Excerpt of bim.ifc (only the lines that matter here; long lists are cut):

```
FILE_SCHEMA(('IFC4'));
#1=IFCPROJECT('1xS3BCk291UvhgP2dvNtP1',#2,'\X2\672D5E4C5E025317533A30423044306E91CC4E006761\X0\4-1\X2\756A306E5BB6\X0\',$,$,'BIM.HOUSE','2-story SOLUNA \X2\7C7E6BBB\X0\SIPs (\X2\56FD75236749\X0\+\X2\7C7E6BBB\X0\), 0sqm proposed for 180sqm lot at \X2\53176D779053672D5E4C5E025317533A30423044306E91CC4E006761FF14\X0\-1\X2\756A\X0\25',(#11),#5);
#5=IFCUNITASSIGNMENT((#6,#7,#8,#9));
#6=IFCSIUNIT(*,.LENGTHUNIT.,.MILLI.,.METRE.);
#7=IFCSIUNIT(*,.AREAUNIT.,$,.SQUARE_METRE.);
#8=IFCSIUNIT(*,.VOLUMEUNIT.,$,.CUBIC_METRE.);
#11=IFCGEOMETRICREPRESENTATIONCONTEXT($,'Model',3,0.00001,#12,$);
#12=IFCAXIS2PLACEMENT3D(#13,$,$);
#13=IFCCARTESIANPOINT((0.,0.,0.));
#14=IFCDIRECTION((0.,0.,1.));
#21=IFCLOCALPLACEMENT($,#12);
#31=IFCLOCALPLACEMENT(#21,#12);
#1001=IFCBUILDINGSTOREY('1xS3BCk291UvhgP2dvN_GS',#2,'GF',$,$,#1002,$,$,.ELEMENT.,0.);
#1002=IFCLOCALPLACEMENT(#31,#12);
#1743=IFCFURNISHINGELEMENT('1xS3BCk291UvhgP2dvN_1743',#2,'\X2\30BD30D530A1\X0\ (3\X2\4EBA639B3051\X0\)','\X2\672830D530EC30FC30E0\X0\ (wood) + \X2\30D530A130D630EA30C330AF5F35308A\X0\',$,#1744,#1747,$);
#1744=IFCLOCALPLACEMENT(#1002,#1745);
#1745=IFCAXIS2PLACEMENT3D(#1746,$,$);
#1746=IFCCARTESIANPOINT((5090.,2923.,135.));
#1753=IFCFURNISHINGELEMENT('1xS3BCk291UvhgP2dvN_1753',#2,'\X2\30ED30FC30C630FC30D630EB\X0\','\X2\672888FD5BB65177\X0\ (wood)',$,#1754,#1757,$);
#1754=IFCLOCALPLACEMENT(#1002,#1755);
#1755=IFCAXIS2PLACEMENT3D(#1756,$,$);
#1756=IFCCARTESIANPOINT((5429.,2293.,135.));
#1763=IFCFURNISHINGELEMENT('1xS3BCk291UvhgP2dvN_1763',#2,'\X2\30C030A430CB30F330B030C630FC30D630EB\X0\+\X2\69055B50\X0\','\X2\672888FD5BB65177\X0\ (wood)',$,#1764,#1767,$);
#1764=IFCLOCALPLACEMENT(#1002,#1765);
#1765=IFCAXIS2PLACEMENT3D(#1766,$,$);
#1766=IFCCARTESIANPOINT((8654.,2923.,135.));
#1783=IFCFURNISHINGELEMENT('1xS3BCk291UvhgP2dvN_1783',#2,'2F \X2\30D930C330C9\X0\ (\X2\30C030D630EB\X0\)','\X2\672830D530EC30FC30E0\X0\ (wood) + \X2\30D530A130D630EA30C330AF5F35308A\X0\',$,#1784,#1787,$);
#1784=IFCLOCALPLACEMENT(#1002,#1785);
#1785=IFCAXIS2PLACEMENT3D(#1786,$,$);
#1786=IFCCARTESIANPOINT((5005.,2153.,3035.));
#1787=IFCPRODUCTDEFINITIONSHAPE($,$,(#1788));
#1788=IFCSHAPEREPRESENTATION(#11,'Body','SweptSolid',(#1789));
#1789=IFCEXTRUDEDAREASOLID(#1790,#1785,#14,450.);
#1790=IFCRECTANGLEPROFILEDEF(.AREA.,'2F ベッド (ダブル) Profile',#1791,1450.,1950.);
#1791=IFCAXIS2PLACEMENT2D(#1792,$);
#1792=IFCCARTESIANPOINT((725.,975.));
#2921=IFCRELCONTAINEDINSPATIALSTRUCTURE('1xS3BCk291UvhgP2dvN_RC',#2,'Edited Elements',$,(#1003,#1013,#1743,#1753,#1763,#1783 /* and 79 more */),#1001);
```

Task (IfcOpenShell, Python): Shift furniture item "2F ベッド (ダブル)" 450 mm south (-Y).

```python
import ifcopenshell
import ifcopenshell.api.geometry
import ifcopenshell.util.placement
import ifcopenshell.util.unit

model = ifcopenshell.open("bim.ifc")
unit_scale = ifcopenshell.util.unit.calculate_unit_scale(model)

item = model.by_id(1783)
matrix = ifcopenshell.util.placement.get_local_placement(item.ObjectPlacement)
matrix[1, 3] -= 0.45 / unit_scale
ifcopenshell.api.geometry.edit_object_placement(model, product=item, matrix=matrix, is_si=False)

print(ifcopenshell.util.placement.get_local_placement(item.ObjectPlacement).round(3) + 0.0)

model.write("bim_rev.ifc")
```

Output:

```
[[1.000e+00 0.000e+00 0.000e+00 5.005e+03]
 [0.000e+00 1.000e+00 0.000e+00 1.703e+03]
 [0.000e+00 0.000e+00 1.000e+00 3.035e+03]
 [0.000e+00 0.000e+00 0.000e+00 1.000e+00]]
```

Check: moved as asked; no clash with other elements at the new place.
